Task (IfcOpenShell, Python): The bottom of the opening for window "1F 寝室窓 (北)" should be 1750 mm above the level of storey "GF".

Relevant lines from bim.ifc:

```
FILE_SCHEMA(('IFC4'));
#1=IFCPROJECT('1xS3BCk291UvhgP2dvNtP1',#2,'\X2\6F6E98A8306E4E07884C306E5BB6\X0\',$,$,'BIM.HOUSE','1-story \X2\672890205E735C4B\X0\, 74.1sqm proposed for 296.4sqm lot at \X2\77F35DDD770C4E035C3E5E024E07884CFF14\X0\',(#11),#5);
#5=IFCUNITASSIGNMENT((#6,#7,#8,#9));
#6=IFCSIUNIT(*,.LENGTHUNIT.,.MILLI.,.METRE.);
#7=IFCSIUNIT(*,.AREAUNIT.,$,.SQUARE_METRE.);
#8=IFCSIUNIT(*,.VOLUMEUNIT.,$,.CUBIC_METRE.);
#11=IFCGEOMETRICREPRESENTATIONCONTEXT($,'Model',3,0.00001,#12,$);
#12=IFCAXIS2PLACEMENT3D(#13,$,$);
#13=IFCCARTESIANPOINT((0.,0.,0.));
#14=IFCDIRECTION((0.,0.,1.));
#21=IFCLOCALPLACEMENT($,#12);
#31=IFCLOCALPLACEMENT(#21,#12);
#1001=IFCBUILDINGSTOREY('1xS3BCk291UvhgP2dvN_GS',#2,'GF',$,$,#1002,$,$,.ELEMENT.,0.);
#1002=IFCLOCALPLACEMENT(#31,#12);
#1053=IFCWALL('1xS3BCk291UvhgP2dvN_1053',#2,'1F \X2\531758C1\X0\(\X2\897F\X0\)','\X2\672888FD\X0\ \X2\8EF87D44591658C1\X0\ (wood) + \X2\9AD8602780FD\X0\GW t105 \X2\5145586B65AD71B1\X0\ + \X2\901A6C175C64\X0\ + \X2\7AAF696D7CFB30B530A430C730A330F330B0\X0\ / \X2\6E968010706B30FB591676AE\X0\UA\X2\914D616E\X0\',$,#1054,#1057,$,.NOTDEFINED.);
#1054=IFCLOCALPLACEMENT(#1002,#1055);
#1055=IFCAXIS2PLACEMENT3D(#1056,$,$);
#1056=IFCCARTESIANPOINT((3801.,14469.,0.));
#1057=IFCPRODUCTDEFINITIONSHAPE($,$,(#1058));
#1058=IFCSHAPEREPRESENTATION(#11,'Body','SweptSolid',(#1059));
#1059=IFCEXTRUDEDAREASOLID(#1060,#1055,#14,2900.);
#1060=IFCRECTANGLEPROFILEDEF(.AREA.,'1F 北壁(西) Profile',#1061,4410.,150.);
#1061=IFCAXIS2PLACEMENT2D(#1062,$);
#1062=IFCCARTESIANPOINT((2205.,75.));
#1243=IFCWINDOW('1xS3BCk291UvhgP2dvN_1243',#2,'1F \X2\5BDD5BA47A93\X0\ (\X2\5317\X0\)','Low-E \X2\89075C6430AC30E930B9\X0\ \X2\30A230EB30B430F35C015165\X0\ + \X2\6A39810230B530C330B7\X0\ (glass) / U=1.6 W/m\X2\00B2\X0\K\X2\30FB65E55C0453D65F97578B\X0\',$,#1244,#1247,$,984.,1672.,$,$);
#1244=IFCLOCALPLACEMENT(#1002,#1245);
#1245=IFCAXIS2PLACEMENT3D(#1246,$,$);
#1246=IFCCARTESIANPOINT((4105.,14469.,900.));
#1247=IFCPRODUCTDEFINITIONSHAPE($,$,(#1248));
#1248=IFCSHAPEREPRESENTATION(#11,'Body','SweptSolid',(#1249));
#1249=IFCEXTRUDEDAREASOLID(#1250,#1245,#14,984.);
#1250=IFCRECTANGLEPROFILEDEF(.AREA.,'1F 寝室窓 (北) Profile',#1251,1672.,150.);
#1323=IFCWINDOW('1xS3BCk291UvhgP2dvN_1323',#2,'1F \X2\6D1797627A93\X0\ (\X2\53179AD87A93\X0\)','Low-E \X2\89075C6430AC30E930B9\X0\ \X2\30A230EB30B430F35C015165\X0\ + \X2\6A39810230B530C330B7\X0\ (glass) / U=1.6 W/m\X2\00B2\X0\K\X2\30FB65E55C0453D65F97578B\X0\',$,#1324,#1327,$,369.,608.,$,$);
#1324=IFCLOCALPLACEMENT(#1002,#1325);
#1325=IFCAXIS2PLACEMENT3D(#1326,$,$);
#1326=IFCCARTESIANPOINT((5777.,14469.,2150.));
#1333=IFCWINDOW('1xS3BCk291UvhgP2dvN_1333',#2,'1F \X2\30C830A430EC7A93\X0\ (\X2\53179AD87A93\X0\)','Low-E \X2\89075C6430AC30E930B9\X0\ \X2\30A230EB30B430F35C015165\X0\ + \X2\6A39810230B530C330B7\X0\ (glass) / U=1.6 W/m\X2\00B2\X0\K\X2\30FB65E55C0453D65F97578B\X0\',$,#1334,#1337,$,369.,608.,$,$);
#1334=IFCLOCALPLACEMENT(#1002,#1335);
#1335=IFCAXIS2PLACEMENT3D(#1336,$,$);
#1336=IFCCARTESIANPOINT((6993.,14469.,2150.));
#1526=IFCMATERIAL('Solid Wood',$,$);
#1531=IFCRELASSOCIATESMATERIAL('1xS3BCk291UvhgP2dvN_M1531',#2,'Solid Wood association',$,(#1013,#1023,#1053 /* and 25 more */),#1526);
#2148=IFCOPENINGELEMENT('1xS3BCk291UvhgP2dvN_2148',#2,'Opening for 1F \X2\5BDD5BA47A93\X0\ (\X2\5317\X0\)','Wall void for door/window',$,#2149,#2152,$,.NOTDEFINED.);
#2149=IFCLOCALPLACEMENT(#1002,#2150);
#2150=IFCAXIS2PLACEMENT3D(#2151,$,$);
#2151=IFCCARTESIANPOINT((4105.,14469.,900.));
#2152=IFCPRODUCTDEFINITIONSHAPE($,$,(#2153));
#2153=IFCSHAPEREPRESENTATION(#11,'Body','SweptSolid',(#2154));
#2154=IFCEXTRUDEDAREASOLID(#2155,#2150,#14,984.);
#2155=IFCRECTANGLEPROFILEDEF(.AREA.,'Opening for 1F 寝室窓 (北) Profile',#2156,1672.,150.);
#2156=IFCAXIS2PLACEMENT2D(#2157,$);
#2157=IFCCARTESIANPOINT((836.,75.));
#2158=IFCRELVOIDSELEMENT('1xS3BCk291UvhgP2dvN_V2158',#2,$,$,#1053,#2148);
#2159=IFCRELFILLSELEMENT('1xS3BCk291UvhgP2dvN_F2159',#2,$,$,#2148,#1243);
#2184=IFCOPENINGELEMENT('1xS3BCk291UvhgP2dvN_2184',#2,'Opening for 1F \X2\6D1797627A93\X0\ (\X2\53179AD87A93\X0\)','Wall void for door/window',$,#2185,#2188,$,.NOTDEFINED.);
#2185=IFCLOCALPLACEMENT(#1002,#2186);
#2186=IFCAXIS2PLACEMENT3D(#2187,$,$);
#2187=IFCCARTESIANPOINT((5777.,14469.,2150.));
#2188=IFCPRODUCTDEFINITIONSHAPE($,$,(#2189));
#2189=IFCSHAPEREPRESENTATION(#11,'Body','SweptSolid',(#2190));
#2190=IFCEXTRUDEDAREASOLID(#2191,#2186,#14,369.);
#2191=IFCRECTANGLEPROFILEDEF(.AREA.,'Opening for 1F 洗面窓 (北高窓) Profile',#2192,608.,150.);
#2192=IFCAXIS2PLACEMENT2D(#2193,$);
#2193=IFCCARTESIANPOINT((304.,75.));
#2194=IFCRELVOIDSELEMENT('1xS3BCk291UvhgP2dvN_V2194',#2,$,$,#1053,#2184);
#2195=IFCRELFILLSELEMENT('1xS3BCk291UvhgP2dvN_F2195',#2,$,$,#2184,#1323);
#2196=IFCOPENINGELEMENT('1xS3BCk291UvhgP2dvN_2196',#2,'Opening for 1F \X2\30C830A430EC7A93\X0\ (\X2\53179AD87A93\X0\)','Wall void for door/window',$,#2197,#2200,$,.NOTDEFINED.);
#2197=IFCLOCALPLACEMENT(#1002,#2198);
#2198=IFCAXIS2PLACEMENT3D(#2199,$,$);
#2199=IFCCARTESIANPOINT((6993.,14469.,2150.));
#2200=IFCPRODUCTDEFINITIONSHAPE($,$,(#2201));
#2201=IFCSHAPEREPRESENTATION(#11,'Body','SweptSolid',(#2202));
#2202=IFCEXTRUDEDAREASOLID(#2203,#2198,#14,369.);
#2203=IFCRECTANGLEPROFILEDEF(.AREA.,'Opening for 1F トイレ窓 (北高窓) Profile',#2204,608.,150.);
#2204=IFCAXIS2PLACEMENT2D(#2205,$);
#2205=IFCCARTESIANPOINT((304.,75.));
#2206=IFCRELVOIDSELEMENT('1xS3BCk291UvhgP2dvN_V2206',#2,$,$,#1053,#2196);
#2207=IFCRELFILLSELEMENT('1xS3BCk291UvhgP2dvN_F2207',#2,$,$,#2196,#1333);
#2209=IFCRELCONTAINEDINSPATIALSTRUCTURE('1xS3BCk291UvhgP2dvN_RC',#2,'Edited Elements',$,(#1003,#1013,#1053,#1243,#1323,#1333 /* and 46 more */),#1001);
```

```python
import numpy as np
import ifcopenshell
import ifcopenshell.api.geometry
import ifcopenshell.geom
import ifcopenshell.util.element
import ifcopenshell.util.placement
import ifcopenshell.util.shape
import ifcopenshell.util.unit

model = ifcopenshell.open("bim.ifc")
unit_scale = ifcopenshell.util.unit.calculate_unit_scale(model)

window = model.by_guid("1xS3BCk291UvhgP2dvN_1243")
opening = window.FillsVoids[0].RelatingOpeningElement
storey = ifcopenshell.util.element.get_container(window, ifc_class="IfcBuildingStorey")
level = ifcopenshell.util.placement.get_local_placement(storey.ObjectPlacement)[2, 3]

# The opening's origin need not be at the sill, so measure its lowest point.
shape = ifcopenshell.geom.create_shape(ifcopenshell.geom.settings(), opening)
bottom = ifcopenshell.util.shape.get_shape_bottom_elevation(shape, shape.geometry) / unit_scale
dz = level + 1750.0 - bottom

shift = np.array([0.0, 0.0, dz])
# The window is not placed relative to its opening, so move both.
for product in (opening, window):
    matrix = ifcopenshell.util.placement.get_local_placement(product.ObjectPlacement)
    matrix[:3, 3] += shift
    ifcopenshell.api.geometry.edit_object_placement(model, product=product, matrix=matrix, is_si=False)

print(f"moved by {dz * unit_scale:+.3f} m")

model.write("bim_rev.ifc")
```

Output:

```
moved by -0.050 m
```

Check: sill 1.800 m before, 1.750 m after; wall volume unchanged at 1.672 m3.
